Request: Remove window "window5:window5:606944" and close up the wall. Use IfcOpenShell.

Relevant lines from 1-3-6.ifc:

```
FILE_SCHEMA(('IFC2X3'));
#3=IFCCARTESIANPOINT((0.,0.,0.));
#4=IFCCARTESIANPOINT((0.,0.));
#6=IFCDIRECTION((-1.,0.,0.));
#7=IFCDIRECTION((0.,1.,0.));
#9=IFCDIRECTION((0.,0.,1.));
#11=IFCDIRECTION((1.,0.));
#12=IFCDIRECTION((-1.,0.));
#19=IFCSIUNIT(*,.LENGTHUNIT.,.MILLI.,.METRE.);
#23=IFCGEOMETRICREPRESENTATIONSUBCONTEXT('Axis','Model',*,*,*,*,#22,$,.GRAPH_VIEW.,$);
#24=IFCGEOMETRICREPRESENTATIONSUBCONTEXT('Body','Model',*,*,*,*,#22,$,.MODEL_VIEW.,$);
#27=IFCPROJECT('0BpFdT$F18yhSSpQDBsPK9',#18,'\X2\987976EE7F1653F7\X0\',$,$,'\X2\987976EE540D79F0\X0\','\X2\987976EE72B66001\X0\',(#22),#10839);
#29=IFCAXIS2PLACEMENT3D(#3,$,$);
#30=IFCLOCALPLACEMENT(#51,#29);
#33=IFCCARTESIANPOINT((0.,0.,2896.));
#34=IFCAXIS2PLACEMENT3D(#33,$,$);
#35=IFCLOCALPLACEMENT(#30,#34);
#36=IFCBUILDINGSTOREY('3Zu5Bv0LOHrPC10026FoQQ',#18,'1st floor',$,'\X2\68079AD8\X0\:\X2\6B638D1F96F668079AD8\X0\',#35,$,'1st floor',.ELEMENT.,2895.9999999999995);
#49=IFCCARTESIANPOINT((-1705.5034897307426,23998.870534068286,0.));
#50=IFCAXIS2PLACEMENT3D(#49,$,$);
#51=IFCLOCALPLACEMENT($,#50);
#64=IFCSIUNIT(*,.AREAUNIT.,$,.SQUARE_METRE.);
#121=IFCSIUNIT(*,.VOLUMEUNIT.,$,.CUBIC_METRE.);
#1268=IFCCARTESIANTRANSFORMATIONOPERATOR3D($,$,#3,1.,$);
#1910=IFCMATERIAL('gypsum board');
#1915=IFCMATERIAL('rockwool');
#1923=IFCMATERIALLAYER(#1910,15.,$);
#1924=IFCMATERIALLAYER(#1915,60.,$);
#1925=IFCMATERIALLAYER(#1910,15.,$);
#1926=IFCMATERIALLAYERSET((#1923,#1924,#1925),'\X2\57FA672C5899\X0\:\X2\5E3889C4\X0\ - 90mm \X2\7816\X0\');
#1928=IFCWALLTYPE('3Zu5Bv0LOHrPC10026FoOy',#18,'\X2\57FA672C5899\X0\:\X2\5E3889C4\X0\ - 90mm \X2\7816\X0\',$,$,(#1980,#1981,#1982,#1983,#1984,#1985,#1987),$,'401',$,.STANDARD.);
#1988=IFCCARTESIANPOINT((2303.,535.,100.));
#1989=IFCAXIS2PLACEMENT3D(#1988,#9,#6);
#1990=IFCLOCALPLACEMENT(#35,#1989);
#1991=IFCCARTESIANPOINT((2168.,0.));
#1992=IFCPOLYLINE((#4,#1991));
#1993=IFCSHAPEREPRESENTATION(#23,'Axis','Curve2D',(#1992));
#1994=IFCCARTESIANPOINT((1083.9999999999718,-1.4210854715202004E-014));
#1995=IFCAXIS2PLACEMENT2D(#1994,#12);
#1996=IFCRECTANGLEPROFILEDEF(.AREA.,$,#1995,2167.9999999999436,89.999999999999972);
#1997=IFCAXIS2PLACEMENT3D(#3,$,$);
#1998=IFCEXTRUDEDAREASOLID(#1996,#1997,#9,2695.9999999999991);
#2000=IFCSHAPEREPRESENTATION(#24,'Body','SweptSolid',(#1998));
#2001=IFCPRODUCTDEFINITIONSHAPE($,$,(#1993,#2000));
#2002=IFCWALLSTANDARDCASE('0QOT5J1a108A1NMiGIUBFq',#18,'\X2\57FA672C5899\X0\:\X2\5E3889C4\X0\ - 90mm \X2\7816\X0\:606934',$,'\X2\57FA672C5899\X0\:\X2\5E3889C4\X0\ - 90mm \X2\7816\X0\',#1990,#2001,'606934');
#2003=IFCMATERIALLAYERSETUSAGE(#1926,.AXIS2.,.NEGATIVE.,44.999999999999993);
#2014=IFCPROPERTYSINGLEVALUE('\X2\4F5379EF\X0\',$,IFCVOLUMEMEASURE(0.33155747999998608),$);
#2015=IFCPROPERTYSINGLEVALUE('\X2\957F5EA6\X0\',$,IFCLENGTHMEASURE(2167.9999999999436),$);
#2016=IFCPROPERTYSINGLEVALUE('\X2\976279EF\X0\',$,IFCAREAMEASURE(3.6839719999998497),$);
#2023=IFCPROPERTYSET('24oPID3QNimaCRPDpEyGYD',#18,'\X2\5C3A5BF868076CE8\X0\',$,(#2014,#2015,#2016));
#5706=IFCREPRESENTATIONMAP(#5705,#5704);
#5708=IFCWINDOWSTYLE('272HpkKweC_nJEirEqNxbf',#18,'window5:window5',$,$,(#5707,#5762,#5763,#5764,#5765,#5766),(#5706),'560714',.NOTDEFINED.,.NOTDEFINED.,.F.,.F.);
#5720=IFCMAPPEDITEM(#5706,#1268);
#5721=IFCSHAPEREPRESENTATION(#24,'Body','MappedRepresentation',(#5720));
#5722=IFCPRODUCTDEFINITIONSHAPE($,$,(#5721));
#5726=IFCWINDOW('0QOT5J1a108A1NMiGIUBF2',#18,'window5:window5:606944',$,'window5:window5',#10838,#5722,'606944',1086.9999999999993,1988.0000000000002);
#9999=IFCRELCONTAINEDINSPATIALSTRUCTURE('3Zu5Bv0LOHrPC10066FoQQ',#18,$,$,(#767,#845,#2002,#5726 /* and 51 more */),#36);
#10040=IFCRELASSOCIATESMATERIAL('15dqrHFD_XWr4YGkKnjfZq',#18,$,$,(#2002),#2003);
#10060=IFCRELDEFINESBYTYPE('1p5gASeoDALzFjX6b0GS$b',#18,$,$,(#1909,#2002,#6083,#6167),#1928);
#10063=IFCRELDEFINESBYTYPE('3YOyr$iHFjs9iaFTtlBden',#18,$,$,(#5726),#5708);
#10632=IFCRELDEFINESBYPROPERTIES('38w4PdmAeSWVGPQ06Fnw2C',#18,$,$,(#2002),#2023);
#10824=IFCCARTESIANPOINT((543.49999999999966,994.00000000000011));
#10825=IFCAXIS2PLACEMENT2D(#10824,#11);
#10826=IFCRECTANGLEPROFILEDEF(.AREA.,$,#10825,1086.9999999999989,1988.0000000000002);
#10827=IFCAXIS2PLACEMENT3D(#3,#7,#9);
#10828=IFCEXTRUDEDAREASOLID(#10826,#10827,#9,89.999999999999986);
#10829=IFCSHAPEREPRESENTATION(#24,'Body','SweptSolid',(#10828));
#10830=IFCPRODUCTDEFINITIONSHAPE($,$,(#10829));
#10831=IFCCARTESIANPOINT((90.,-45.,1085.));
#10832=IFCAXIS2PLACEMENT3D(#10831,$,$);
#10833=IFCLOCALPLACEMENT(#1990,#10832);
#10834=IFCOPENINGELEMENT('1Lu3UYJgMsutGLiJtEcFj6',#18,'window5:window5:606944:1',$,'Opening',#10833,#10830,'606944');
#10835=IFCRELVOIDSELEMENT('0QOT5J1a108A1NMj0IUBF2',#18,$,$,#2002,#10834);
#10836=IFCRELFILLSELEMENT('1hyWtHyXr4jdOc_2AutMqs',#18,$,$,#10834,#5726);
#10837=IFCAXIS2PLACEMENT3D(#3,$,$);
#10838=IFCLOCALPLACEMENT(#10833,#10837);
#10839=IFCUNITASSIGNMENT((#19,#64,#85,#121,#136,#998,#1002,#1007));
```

```python
import ifcopenshell
import ifcopenshell.api.feature
import ifcopenshell.api.pset
import ifcopenshell.api.root
import ifcopenshell.geom
import ifcopenshell.util.element
import ifcopenshell.util.shape
import ifcopenshell.util.unit

model = ifcopenshell.open("1-3-6.ifc")
area_scale = ifcopenshell.util.unit.calculate_unit_scale(model, "AREAUNIT")
volume_scale = ifcopenshell.util.unit.calculate_unit_scale(model, "VOLUMEUNIT")
settings = ifcopenshell.geom.settings()


def volume(element):
    """Net volume in cubic metres, openings subtracted."""
    shape = ifcopenshell.geom.create_shape(settings, element)
    return ifcopenshell.util.shape.get_volume(shape.geometry)


window = model.by_guid("0QOT5J1a108A1NMiGIUBF2")
opening = window.FillsVoids[0].RelatingOpeningElement
wall = opening.VoidsElements[0].RelatingBuildingElement
before = volume(wall)

ifcopenshell.api.root.remove_product(model, product=window)
ifcopenshell.api.feature.remove_feature(model, feature=opening)

after = volume(wall)
thickness = 0.09  # wall thickness in metres

# Update the wall's stored quantities.
pset = model.by_id(ifcopenshell.util.element.get_pset(wall, "尺寸标注", should_inherit=False)["id"])
ifcopenshell.api.pset.edit_pset(model, pset=pset, properties={
    "体积": model.create_entity("IfcVolumeMeasure", after / volume_scale),
    "面积": model.create_entity("IfcAreaMeasure", after / thickness / area_scale),
})

print(f"wall volume {before:.3f} -> {after:.3f} m3")

model.write("1-3-6_updated.ifc")
```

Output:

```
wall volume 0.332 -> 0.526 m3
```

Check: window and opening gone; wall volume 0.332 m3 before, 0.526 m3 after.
